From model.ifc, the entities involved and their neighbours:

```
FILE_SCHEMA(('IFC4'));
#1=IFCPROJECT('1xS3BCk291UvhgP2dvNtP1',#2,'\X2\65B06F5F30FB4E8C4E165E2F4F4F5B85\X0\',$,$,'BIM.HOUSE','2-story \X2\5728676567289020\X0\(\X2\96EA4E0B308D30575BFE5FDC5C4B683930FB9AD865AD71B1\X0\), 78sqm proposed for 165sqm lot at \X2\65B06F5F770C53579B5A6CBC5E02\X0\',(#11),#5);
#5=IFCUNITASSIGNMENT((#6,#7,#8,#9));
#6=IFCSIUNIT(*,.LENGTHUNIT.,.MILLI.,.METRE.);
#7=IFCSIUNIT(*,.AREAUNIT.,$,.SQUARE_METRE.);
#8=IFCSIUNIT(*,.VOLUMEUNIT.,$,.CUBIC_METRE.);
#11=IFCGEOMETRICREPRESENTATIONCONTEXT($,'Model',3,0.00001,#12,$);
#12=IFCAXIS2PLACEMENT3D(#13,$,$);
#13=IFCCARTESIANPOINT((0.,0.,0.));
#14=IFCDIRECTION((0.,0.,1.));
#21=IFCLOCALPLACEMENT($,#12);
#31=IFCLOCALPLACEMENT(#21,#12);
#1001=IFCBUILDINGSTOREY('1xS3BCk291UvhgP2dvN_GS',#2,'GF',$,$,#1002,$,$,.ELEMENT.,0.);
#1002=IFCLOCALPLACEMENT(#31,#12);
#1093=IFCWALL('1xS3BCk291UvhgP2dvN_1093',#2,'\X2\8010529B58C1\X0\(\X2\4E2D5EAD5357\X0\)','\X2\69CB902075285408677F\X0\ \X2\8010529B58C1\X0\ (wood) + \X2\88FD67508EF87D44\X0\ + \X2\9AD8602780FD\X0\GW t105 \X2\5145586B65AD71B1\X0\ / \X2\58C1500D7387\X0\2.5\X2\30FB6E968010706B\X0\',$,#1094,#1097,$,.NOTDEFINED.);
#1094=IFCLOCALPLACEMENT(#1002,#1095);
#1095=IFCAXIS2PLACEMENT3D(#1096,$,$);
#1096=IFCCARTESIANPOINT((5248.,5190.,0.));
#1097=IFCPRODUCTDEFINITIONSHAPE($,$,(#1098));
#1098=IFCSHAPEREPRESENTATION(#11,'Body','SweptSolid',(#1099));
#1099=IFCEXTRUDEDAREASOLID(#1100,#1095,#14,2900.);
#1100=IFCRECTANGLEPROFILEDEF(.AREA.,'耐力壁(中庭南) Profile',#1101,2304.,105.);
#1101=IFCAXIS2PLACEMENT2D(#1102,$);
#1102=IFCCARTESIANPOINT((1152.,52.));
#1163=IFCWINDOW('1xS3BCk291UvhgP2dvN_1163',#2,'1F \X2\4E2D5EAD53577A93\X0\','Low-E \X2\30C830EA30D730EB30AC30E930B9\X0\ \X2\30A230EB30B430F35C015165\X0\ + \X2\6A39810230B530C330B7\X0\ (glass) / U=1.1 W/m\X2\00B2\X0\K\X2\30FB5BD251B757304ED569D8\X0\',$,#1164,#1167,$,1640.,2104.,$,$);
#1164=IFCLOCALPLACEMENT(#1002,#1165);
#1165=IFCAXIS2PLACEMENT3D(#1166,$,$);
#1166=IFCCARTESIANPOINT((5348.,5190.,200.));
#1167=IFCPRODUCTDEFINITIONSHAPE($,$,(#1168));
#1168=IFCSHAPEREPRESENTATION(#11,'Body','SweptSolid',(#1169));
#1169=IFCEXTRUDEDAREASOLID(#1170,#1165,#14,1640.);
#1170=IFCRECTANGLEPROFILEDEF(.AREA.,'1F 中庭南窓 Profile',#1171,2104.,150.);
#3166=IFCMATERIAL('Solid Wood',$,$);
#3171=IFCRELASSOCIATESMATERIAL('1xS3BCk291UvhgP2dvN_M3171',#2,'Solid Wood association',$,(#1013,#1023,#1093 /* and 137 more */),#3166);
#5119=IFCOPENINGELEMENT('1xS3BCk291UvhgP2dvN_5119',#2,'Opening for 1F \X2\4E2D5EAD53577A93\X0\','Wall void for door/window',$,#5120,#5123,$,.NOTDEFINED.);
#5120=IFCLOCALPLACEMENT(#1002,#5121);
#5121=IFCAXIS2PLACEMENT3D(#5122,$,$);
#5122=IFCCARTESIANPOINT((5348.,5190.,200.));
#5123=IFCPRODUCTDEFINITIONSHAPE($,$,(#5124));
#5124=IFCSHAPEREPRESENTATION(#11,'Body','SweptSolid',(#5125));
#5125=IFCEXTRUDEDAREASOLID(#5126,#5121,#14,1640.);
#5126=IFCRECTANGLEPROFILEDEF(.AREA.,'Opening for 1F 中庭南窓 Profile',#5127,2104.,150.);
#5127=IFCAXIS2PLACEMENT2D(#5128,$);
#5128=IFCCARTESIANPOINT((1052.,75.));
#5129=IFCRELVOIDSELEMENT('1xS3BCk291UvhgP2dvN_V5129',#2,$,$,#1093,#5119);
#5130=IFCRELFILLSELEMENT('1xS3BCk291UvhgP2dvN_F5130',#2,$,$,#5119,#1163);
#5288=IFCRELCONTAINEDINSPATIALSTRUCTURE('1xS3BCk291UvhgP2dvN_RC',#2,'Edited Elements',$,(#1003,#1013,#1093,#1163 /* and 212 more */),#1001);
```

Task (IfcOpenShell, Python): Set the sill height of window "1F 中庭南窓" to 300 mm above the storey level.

```python
import numpy as np
import ifcopenshell
import ifcopenshell.api.geometry
import ifcopenshell.geom
import ifcopenshell.util.element
import ifcopenshell.util.placement
import ifcopenshell.util.shape
import ifcopenshell.util.unit

model = ifcopenshell.open("model.ifc")
unit_scale = ifcopenshell.util.unit.calculate_unit_scale(model)

window = model.by_guid("1xS3BCk291UvhgP2dvN_1163")
opening = window.FillsVoids[0].RelatingOpeningElement
storey = ifcopenshell.util.element.get_container(window, ifc_class="IfcBuildingStorey")
level = ifcopenshell.util.placement.get_local_placement(storey.ObjectPlacement)[2, 3]

# The opening's origin need not be at the sill, so measure its lowest point.
shape = ifcopenshell.geom.create_shape(ifcopenshell.geom.settings(), opening)
bottom = ifcopenshell.util.shape.get_shape_bottom_elevation(shape, shape.geometry) / unit_scale
dz = level + 0.3 / unit_scale - bottom

shift = np.array([0.0, 0.0, dz])
# The window is not placed relative to its opening, so move both.
for product in (opening, window):
    matrix = ifcopenshell.util.placement.get_local_placement(product.ObjectPlacement)
    matrix[:3, 3] += shift
    ifcopenshell.api.geometry.edit_object_placement(model, product=product, matrix=matrix, is_si=False)

print(f"moved by {dz * unit_scale:+.3f} m")

model.write("model_edited.ifc")
```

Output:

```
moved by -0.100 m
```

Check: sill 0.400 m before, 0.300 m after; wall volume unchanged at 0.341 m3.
